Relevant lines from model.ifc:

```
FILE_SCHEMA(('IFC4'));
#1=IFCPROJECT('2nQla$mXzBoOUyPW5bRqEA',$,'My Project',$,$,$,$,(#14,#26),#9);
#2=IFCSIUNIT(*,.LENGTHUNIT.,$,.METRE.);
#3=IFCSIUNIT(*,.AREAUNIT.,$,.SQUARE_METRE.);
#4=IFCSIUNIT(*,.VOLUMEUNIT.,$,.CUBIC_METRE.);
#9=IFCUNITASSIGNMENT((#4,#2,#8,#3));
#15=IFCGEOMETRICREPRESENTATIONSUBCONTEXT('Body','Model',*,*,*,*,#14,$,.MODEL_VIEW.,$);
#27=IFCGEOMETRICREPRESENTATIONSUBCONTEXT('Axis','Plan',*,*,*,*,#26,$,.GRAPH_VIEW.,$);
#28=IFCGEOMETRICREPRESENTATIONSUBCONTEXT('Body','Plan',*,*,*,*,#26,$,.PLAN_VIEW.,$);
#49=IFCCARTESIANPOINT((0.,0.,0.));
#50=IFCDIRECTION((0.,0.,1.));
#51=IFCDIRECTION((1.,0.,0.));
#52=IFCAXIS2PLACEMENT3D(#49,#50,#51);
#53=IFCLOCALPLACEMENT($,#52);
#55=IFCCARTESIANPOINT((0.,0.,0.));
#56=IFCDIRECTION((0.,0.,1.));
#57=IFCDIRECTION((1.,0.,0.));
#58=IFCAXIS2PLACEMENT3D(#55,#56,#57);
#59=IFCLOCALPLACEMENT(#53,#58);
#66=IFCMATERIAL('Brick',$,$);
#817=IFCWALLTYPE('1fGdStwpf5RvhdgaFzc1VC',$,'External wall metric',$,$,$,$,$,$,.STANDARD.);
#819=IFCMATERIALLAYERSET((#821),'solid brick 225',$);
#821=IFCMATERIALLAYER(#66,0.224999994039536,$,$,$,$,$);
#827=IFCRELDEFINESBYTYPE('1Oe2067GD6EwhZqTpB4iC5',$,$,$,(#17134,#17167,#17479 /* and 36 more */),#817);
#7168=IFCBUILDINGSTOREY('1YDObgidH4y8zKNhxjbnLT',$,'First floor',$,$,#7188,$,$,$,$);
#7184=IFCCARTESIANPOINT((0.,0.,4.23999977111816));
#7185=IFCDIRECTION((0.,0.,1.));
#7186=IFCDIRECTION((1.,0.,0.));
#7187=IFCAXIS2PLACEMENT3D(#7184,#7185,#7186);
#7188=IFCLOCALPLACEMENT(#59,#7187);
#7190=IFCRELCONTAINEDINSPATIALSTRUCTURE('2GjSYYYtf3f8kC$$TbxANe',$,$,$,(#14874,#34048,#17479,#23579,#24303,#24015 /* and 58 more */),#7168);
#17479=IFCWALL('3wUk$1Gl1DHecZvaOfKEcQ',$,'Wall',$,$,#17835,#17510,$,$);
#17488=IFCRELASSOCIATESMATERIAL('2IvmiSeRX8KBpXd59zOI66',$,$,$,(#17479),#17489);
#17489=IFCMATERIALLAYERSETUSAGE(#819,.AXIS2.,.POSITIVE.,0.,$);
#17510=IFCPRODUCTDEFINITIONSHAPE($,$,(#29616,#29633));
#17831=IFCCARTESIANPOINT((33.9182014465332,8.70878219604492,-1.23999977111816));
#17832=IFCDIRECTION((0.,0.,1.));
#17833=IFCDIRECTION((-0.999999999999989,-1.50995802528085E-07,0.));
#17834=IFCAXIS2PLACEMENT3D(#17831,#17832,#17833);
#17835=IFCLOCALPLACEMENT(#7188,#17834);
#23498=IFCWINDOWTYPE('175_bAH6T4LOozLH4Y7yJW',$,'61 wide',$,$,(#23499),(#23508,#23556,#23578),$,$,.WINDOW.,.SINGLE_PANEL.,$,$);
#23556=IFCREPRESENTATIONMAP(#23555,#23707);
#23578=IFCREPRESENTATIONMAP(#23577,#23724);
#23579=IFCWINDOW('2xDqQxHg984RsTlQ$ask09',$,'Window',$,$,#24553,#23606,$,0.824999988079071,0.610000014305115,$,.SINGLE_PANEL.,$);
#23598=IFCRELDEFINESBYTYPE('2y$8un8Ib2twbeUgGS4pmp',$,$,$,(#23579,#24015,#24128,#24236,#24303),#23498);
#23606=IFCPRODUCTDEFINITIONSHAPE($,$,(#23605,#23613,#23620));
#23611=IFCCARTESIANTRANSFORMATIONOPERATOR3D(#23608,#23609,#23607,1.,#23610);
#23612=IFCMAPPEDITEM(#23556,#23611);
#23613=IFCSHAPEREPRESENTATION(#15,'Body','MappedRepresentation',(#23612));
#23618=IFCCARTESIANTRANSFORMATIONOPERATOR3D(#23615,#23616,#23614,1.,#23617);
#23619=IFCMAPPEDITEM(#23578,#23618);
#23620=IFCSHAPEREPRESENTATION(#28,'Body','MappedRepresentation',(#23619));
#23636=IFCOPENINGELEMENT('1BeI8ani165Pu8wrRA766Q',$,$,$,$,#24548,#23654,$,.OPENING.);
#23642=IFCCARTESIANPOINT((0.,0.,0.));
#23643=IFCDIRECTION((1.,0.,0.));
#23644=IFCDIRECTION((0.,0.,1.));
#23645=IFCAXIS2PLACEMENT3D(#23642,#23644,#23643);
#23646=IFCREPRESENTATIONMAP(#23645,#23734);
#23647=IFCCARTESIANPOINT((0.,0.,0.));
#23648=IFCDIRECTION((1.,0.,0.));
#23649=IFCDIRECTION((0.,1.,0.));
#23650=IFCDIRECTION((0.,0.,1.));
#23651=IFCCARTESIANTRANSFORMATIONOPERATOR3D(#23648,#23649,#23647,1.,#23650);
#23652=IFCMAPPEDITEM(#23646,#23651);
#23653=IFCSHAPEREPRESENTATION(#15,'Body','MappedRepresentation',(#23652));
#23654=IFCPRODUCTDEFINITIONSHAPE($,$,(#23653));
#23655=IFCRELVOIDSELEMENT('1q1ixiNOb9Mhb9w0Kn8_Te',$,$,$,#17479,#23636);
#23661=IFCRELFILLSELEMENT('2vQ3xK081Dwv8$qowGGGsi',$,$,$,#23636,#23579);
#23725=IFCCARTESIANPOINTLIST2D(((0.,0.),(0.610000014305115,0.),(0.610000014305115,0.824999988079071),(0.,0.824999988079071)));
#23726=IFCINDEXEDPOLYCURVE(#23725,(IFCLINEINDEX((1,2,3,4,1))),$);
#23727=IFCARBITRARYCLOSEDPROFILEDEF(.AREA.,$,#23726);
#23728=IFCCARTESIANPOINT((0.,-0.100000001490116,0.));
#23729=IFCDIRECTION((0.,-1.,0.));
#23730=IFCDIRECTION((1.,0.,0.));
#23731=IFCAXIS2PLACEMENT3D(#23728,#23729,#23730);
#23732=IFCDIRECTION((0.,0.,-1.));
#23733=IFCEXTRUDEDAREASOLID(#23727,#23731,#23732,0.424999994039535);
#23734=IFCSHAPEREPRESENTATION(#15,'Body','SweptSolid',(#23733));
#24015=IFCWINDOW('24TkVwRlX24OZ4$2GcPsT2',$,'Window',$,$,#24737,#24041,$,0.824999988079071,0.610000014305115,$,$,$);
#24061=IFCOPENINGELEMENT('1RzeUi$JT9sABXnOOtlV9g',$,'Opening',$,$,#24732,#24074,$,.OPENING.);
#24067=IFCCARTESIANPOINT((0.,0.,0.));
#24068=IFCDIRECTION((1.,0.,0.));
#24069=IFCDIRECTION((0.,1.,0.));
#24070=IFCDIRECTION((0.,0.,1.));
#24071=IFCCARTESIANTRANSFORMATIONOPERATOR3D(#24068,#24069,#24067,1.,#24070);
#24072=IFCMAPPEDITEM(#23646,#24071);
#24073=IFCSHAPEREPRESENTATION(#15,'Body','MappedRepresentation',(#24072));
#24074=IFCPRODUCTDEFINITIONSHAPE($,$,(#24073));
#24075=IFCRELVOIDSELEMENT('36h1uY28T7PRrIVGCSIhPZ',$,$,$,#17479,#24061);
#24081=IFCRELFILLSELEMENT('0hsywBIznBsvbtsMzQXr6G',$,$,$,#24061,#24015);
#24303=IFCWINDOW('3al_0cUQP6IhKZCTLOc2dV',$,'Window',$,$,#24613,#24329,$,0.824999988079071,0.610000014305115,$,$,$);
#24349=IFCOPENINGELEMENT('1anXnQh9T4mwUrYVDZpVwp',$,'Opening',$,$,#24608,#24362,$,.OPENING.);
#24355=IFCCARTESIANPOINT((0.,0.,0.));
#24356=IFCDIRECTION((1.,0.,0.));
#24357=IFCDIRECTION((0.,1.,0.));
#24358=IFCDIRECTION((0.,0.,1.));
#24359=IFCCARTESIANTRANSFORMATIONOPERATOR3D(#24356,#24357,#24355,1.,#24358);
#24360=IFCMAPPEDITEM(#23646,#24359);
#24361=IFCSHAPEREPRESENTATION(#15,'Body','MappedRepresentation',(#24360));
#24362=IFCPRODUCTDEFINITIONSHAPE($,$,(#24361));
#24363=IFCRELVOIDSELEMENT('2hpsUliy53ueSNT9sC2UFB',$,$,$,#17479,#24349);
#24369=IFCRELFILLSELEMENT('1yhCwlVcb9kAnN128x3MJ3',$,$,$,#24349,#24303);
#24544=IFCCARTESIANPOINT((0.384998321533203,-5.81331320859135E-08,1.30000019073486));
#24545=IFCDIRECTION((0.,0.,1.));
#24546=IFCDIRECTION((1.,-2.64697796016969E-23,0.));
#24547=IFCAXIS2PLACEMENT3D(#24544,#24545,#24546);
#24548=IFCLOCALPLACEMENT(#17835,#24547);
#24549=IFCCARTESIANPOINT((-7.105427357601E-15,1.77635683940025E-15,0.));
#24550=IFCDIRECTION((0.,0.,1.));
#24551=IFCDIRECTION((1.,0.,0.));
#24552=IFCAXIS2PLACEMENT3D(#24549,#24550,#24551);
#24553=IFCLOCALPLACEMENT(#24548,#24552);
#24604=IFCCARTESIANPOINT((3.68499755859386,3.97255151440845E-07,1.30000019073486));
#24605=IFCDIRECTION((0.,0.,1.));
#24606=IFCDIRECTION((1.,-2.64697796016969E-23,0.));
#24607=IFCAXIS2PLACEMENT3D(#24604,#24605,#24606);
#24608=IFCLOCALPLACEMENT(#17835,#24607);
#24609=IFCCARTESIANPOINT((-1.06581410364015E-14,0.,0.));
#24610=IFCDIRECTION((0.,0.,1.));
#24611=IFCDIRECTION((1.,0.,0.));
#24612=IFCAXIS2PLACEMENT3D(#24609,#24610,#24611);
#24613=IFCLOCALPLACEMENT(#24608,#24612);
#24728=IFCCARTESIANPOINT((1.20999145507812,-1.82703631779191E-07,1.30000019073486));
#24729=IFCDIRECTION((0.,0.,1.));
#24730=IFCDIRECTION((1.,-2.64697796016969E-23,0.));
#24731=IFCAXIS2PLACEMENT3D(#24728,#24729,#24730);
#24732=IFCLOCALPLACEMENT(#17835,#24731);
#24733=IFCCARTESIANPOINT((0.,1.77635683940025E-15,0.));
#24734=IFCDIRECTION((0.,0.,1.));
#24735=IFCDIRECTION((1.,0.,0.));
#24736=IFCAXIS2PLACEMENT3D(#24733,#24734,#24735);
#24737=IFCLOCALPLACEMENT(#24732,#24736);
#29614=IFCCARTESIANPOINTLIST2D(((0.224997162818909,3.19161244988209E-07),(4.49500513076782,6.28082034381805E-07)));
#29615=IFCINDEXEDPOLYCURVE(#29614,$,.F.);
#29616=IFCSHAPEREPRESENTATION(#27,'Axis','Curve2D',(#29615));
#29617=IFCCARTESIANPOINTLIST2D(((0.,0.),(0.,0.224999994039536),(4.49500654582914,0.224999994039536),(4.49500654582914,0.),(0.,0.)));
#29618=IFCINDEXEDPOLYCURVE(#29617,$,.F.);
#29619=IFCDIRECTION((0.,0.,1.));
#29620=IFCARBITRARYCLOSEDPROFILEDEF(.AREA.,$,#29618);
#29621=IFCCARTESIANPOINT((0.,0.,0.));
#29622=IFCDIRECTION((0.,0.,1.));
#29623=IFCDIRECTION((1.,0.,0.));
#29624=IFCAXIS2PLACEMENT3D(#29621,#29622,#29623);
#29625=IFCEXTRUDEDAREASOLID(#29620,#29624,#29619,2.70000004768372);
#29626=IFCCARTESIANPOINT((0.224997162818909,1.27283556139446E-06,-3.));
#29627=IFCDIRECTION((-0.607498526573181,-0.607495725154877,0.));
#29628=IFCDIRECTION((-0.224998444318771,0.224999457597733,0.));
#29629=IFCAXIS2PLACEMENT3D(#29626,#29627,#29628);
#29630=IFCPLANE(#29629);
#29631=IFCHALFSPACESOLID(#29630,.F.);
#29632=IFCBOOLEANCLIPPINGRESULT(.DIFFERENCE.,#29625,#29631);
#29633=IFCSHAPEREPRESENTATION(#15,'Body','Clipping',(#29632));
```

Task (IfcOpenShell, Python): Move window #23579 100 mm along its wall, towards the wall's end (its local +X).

```python
import ifcopenshell
import ifcopenshell.api.geometry
import ifcopenshell.util.placement
import ifcopenshell.util.unit

model = ifcopenshell.open("model.ifc")
unit_scale = ifcopenshell.util.unit.calculate_unit_scale(model)

window = model.by_guid("2xDqQxHg984RsTlQ$ask09")
opening = window.FillsVoids[0].RelatingOpeningElement
wall = opening.VoidsElements[0].RelatingBuildingElement

wall_matrix = ifcopenshell.util.placement.get_local_placement(wall.ObjectPlacement)
shift = wall_matrix[:3, 0] * 0.1 / unit_scale
before = ifcopenshell.util.placement.get_local_placement(window.ObjectPlacement)[:3, 3].copy()

# The window is placed relative to its opening, so it follows when the opening moves.
matrix = ifcopenshell.util.placement.get_local_placement(opening.ObjectPlacement)
matrix[:3, 3] += shift
ifcopenshell.api.geometry.edit_object_placement(
    model, product=opening, matrix=matrix, is_si=False, should_transform_children=True
)

after = ifcopenshell.util.placement.get_local_placement(window.ObjectPlacement)[:3, 3]
print("window moved by", (after - before).round(3) + 0.0)

model.write("model_rev.ifc")
```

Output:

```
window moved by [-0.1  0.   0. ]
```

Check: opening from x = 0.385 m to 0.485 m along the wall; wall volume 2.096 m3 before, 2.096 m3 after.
